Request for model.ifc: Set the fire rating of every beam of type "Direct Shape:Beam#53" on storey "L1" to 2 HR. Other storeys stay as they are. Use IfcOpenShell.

First a look at what the model holds.

```python
import ifcopenshell
import ifcopenshell.util.element

model = ifcopenshell.open("model.ifc")
print(model.schema)
storey = next(s for s in model.by_type("IfcBuildingStorey") if s.Name == "L1")
beams = [e for e in ifcopenshell.util.element.get_decomposition(storey) if e.is_a("IfcBeam")]
seen = {}
for e in beams:
    element_type = ifcopenshell.util.element.get_type(e)
    key = (element_type.Name if element_type != e and element_type else None, ifcopenshell.util.element.get_pset(e, "Pset_BeamCommon", "FireRating"))
    seen[key] = seen.get(key, 0) + 1
for (name, value), count in sorted(seen.items(), key=str):
    print(count, "x", name, "|", value)
```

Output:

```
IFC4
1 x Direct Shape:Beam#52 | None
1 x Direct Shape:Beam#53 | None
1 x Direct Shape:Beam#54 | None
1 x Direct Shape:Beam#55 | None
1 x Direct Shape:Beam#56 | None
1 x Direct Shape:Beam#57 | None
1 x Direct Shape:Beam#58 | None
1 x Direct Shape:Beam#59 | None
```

```python
import ifcopenshell
import ifcopenshell.api.pset
import ifcopenshell.util.element

model = ifcopenshell.open("model.ifc")

storey = next(s for s in model.by_type("IfcBuildingStorey") if s.Name == "L1")
beams = [e for e in ifcopenshell.util.element.get_decomposition(storey) if e.is_a("IfcBeam")]

count = 0
for e in beams:
    element_type = ifcopenshell.util.element.get_type(e)
    if element_type in (None, e) or element_type.Name != "Direct Shape:Beam#53":
        continue
    # add_pset returns the element's existing set when there is one.
    pset = ifcopenshell.api.pset.add_pset(model, product=e, name="Pset_BeamCommon")
    ifcopenshell.api.pset.edit_pset(model, pset=pset, properties={"FireRating": "2 HR"})
    count += 1

print(count, "beams updated")

model.write("model_updated.ifc")
```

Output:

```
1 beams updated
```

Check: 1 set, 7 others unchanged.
